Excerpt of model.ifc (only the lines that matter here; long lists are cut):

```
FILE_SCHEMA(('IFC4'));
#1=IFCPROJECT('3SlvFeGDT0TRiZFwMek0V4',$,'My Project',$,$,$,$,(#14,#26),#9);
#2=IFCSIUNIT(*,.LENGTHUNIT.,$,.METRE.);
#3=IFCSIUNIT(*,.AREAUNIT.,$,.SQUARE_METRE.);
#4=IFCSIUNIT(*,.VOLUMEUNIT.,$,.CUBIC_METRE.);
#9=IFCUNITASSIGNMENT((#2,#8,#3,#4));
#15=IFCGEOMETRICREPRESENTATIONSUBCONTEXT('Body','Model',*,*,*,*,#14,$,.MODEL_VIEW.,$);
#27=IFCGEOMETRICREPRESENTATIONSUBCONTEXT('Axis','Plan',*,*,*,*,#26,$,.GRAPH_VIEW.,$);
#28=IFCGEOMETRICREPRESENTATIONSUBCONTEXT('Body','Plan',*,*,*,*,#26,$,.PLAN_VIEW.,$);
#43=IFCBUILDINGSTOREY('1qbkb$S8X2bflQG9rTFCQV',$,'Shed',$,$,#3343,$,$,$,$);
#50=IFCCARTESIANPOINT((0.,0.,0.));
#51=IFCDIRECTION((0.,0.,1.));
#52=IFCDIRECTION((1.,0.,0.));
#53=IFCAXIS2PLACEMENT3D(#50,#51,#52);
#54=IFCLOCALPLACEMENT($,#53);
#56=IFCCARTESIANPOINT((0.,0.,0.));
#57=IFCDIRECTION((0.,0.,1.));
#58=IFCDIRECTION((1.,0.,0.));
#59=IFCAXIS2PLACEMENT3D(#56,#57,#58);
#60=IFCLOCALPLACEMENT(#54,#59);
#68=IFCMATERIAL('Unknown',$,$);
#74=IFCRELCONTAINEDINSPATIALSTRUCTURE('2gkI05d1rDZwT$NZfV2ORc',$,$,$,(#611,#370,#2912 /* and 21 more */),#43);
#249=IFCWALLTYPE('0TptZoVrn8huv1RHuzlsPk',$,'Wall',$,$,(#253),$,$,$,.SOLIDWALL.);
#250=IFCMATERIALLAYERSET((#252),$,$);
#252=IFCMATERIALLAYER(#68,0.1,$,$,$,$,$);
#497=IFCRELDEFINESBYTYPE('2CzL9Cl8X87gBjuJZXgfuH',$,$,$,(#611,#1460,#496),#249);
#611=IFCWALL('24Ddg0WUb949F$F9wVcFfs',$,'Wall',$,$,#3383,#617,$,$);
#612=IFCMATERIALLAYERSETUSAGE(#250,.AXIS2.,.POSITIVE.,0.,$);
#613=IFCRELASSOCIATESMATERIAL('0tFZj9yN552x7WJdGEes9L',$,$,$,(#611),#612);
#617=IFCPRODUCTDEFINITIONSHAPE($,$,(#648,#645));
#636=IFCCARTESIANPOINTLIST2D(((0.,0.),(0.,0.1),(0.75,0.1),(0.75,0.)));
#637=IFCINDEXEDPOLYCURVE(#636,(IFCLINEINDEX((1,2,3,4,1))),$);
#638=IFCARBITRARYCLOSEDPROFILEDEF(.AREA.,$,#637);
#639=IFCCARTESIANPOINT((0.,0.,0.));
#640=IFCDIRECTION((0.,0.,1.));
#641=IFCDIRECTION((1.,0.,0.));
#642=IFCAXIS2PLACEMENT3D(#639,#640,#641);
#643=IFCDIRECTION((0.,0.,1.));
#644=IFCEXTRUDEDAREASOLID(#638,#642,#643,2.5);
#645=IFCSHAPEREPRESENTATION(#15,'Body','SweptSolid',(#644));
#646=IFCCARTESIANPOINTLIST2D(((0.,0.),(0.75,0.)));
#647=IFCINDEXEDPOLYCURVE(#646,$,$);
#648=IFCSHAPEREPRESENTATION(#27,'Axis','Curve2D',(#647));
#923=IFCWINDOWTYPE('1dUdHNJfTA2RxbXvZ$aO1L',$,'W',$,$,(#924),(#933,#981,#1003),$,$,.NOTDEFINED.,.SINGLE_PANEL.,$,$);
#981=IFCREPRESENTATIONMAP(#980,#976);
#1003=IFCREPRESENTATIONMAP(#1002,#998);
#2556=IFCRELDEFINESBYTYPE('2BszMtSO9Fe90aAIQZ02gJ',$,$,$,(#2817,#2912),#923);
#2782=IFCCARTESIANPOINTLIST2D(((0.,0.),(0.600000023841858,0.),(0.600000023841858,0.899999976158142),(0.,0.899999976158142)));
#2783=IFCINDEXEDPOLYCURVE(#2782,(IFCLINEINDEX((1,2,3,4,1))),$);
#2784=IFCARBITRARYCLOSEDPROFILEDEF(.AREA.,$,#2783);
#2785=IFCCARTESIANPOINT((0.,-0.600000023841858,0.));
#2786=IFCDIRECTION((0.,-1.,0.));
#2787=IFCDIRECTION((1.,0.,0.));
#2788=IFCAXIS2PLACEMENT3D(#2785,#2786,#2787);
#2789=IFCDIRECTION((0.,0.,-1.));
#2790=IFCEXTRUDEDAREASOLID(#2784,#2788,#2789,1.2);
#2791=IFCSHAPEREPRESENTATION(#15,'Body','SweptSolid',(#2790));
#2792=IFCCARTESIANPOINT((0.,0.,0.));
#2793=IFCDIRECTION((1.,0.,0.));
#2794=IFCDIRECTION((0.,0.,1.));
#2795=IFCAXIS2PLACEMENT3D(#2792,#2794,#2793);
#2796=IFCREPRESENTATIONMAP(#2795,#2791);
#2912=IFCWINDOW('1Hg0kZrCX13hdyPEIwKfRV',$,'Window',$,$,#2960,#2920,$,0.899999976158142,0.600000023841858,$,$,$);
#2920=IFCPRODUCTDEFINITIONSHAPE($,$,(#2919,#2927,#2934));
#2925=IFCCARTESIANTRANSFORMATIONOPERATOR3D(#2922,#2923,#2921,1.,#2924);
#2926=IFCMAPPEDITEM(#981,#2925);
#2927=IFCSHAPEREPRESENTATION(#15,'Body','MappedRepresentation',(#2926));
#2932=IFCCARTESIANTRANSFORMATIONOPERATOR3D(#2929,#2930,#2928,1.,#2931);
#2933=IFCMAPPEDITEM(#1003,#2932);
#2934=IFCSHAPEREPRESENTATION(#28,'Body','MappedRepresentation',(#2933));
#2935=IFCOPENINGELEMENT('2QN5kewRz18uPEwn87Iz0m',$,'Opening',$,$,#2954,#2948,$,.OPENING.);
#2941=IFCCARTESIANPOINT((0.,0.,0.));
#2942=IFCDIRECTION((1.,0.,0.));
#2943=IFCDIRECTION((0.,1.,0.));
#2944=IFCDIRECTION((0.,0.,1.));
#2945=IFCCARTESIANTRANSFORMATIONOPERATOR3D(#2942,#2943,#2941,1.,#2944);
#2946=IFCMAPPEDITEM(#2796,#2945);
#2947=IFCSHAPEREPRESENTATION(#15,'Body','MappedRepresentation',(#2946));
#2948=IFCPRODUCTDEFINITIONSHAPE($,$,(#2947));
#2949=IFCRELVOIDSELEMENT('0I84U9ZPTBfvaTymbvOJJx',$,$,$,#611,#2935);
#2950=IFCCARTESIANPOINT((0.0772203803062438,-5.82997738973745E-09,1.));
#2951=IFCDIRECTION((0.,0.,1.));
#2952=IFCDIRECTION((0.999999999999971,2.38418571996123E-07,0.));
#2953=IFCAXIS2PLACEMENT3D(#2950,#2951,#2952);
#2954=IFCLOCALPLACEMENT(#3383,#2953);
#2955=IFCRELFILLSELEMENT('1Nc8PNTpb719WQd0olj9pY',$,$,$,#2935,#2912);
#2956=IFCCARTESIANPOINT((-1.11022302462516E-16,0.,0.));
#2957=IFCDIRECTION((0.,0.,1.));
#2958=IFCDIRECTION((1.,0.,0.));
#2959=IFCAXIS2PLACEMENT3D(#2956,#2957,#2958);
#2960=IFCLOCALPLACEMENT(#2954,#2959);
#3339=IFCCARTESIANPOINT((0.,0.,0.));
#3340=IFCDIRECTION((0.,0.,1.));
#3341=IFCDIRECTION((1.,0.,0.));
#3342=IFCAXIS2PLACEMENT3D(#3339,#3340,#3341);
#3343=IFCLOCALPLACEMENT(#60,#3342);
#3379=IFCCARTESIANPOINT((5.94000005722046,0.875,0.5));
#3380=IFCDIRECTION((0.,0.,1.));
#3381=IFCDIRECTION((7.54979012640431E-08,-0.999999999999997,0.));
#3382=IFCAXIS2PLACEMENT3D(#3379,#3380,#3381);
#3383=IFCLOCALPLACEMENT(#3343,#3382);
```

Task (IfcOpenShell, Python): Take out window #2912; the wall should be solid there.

```python
import ifcopenshell
import ifcopenshell.api.feature
import ifcopenshell.api.root
import ifcopenshell.geom
import ifcopenshell.util.shape

model = ifcopenshell.open("model.ifc")
settings = ifcopenshell.geom.settings()


def volume(element):
    """Net volume in cubic metres, openings subtracted."""
    shape = ifcopenshell.geom.create_shape(settings, element)
    return ifcopenshell.util.shape.get_volume(shape.geometry)


window = model.by_guid("1Hg0kZrCX13hdyPEIwKfRV")
opening = window.FillsVoids[0].RelatingOpeningElement
wall = opening.VoidsElements[0].RelatingBuildingElement
before = volume(wall)

ifcopenshell.api.root.remove_product(model, product=window)
ifcopenshell.api.feature.remove_feature(model, feature=opening)

after = volume(wall)

print(f"wall volume {before:.3f} -> {after:.3f} m3")

model.write("model-out.ifc")
```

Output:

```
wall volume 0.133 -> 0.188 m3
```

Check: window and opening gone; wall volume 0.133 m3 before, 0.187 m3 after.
